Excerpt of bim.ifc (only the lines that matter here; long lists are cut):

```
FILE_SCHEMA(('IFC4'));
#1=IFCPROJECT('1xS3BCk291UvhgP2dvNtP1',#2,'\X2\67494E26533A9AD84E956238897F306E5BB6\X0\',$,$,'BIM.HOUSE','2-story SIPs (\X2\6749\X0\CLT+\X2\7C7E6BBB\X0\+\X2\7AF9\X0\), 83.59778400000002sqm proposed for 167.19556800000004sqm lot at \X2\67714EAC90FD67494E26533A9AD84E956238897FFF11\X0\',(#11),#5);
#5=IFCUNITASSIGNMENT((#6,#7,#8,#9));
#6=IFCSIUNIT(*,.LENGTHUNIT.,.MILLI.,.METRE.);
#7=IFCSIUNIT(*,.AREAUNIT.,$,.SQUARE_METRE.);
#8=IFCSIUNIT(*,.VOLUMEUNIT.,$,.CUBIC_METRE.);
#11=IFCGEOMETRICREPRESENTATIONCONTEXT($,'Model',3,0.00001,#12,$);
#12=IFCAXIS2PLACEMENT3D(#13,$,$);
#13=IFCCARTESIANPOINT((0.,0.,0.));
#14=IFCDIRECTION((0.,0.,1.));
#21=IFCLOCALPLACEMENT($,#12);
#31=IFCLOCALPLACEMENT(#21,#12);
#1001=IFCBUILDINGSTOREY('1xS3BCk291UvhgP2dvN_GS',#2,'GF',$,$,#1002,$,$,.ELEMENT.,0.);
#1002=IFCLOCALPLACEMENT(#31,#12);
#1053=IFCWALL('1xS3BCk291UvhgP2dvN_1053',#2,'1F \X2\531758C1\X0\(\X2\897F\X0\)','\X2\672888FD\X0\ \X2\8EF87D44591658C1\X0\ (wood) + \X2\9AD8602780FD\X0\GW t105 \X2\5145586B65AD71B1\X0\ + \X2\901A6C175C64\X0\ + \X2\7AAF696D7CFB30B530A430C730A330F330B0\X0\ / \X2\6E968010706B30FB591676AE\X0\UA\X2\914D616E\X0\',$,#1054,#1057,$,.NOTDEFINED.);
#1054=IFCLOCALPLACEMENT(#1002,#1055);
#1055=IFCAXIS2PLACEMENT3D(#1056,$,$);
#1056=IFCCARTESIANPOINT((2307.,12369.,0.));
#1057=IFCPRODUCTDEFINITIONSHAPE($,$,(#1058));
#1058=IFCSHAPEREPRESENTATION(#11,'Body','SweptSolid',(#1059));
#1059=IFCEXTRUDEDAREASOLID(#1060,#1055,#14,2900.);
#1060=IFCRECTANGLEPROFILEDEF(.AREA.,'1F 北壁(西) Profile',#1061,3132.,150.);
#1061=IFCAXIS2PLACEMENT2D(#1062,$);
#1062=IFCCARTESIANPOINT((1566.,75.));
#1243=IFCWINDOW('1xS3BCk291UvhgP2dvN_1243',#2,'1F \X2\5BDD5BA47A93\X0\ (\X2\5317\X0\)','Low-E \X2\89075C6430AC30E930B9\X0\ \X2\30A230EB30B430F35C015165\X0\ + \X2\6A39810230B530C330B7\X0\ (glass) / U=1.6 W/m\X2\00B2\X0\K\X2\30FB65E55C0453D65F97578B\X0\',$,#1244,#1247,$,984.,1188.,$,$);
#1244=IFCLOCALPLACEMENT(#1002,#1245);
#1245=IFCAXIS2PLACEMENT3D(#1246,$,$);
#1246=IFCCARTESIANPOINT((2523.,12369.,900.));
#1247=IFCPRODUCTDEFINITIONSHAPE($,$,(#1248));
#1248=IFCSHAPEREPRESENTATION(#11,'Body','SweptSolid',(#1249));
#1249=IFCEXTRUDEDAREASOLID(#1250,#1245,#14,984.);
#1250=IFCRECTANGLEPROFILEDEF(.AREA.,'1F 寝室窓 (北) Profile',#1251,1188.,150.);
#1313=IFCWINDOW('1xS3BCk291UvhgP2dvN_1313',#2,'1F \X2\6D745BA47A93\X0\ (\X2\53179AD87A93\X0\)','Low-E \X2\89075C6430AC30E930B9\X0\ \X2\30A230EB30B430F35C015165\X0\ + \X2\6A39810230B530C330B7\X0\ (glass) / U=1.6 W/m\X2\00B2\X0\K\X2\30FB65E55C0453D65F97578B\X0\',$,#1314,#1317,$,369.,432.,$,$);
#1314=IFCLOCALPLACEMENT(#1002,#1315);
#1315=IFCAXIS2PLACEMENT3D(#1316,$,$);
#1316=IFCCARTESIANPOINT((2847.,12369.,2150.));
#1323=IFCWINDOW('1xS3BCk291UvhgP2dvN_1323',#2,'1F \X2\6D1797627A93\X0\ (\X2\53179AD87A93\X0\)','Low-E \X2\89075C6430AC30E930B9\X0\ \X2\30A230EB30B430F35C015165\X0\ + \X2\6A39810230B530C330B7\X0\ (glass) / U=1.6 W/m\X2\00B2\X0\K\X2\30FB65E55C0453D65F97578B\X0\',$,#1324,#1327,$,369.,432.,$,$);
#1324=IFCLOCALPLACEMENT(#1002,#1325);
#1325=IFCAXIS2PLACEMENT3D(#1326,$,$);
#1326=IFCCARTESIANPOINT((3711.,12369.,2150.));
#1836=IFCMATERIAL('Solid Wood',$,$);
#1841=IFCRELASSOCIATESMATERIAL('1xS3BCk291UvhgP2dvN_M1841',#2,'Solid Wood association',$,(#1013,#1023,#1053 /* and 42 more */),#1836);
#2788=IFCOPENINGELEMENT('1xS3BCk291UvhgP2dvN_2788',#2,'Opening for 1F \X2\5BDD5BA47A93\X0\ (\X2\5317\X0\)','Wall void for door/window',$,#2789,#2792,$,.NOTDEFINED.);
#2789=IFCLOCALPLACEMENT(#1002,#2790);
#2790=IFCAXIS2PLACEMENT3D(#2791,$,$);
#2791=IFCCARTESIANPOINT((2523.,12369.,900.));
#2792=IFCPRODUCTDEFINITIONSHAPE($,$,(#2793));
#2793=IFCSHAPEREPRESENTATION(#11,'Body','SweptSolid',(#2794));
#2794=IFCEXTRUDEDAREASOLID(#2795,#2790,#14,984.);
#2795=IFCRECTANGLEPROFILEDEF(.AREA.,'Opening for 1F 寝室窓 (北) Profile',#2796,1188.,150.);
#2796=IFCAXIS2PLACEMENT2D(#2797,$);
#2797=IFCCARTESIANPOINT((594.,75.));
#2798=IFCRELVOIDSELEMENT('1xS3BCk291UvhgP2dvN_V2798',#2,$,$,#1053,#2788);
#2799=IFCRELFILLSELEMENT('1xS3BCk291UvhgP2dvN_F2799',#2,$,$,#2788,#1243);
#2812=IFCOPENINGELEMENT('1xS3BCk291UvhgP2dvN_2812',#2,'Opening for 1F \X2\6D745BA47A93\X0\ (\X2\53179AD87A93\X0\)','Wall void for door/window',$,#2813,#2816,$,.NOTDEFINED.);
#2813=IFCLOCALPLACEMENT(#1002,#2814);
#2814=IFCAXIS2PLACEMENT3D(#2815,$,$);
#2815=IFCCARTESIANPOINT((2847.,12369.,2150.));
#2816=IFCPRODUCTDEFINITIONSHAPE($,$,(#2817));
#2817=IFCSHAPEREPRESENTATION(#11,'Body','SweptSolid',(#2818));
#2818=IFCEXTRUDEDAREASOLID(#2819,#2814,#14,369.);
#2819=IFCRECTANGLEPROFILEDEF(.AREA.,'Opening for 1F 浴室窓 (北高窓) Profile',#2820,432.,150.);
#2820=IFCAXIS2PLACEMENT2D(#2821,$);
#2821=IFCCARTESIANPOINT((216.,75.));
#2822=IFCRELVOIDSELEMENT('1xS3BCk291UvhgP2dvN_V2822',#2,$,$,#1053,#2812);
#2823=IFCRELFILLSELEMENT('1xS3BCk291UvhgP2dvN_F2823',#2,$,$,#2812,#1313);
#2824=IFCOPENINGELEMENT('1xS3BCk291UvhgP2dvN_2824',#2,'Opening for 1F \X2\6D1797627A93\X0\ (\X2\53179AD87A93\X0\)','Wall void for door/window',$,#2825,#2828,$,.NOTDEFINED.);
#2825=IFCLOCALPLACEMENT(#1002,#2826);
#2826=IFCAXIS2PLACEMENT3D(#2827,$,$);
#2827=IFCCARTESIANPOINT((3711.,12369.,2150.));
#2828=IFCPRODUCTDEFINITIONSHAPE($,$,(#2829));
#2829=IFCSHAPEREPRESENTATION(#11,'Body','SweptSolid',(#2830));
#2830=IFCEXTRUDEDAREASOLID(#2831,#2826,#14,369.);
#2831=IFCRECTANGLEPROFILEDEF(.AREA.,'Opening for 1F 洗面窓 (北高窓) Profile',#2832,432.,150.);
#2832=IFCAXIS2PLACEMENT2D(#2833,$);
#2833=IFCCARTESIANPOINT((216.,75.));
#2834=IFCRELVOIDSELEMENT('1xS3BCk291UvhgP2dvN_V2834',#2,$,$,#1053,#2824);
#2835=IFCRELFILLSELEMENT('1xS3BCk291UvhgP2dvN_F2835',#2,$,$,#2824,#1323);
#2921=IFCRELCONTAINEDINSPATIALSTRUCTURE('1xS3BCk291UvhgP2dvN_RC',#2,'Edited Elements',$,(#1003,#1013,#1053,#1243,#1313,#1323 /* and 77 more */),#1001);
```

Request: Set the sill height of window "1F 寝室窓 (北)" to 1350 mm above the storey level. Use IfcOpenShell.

```python
import numpy as np
import ifcopenshell
import ifcopenshell.api.geometry
import ifcopenshell.geom
import ifcopenshell.util.element
import ifcopenshell.util.placement
import ifcopenshell.util.shape
import ifcopenshell.util.unit

model = ifcopenshell.open("bim.ifc")
unit_scale = ifcopenshell.util.unit.calculate_unit_scale(model)

window = model.by_guid("1xS3BCk291UvhgP2dvN_1243")
opening = window.FillsVoids[0].RelatingOpeningElement
storey = ifcopenshell.util.element.get_container(window, ifc_class="IfcBuildingStorey")
level = ifcopenshell.util.placement.get_local_placement(storey.ObjectPlacement)[2, 3]

# The opening's origin need not be at the sill, so measure its lowest point.
shape = ifcopenshell.geom.create_shape(ifcopenshell.geom.settings(), opening)
bottom = ifcopenshell.util.shape.get_shape_bottom_elevation(shape, shape.geometry) / unit_scale
dz = level + 1350.0 - bottom

shift = np.array([0.0, 0.0, dz])
# The window is not placed relative to its opening, so move both.
for product in (opening, window):
    matrix = ifcopenshell.util.placement.get_local_placement(product.ObjectPlacement)
    matrix[:3, 3] += shift
    ifcopenshell.api.geometry.edit_object_placement(model, product=product, matrix=matrix, is_si=False)

print(f"moved by {dz * unit_scale:+.3f} m")

model.write("bim-out.ifc")
```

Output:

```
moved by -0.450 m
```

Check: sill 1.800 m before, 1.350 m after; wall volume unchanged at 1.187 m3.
